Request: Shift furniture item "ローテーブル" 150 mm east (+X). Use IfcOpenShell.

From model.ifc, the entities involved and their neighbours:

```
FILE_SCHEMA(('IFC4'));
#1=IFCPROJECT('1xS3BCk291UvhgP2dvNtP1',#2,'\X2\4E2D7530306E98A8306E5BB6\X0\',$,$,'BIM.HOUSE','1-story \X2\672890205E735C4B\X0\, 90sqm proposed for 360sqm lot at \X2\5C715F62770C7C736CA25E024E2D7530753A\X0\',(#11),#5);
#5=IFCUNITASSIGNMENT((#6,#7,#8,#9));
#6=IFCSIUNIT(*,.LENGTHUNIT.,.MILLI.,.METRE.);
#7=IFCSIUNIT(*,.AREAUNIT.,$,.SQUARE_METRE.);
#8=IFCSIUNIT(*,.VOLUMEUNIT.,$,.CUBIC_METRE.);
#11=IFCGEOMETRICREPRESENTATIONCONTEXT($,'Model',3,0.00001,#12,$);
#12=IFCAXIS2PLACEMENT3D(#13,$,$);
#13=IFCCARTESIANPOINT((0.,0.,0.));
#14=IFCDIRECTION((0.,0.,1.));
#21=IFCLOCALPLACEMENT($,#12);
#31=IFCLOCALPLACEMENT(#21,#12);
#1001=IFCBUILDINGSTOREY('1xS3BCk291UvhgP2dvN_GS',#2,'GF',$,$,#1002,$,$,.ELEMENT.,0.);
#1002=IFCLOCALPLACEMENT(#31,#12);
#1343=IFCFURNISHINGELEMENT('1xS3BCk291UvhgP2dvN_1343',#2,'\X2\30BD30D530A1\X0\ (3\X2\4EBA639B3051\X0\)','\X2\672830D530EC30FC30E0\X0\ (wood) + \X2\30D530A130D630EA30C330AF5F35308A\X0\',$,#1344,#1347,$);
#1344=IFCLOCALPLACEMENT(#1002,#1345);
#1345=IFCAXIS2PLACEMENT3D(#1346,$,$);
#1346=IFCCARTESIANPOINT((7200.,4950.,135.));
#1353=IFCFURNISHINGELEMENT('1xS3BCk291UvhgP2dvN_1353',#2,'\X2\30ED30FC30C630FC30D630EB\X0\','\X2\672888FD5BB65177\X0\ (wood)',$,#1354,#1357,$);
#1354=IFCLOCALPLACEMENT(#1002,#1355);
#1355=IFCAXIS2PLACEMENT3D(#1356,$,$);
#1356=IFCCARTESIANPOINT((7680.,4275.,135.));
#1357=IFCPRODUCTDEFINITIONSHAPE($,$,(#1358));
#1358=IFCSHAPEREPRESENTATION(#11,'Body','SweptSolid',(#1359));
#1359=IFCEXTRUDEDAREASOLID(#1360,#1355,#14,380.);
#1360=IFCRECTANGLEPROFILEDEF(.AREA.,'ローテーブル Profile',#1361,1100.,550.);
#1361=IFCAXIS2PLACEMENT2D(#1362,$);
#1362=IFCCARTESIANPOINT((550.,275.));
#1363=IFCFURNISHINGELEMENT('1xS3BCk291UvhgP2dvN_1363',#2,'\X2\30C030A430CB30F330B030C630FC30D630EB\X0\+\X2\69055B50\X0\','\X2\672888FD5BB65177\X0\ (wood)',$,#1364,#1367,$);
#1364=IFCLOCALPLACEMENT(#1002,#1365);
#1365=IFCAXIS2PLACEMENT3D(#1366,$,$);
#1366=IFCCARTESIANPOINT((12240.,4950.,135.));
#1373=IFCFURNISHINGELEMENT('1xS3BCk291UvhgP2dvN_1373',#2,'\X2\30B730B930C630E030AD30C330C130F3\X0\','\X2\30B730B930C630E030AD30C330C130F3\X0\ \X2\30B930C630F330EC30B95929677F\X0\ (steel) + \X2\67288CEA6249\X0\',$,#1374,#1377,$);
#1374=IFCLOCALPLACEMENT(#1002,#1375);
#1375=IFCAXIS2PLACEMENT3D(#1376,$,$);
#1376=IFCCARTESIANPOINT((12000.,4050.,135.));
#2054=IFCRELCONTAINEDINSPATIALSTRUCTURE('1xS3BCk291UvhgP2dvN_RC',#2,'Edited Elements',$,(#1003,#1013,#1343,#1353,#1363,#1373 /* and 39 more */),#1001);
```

```python
import ifcopenshell
import ifcopenshell.api.geometry
import ifcopenshell.util.placement

model = ifcopenshell.open("model.ifc")

item = model.by_guid("1xS3BCk291UvhgP2dvN_1353")
matrix = ifcopenshell.util.placement.get_local_placement(item.ObjectPlacement)
matrix[0, 3] += 150.0
ifcopenshell.api.geometry.edit_object_placement(model, product=item, matrix=matrix, is_si=False)

print(ifcopenshell.util.placement.get_local_placement(item.ObjectPlacement).round(3) + 0.0)

model.write("model_rev.ifc")
```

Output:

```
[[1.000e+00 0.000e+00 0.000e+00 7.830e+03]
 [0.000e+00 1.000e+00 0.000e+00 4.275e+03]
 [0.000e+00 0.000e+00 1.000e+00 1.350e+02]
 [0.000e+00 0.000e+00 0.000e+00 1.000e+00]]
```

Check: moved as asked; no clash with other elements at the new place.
